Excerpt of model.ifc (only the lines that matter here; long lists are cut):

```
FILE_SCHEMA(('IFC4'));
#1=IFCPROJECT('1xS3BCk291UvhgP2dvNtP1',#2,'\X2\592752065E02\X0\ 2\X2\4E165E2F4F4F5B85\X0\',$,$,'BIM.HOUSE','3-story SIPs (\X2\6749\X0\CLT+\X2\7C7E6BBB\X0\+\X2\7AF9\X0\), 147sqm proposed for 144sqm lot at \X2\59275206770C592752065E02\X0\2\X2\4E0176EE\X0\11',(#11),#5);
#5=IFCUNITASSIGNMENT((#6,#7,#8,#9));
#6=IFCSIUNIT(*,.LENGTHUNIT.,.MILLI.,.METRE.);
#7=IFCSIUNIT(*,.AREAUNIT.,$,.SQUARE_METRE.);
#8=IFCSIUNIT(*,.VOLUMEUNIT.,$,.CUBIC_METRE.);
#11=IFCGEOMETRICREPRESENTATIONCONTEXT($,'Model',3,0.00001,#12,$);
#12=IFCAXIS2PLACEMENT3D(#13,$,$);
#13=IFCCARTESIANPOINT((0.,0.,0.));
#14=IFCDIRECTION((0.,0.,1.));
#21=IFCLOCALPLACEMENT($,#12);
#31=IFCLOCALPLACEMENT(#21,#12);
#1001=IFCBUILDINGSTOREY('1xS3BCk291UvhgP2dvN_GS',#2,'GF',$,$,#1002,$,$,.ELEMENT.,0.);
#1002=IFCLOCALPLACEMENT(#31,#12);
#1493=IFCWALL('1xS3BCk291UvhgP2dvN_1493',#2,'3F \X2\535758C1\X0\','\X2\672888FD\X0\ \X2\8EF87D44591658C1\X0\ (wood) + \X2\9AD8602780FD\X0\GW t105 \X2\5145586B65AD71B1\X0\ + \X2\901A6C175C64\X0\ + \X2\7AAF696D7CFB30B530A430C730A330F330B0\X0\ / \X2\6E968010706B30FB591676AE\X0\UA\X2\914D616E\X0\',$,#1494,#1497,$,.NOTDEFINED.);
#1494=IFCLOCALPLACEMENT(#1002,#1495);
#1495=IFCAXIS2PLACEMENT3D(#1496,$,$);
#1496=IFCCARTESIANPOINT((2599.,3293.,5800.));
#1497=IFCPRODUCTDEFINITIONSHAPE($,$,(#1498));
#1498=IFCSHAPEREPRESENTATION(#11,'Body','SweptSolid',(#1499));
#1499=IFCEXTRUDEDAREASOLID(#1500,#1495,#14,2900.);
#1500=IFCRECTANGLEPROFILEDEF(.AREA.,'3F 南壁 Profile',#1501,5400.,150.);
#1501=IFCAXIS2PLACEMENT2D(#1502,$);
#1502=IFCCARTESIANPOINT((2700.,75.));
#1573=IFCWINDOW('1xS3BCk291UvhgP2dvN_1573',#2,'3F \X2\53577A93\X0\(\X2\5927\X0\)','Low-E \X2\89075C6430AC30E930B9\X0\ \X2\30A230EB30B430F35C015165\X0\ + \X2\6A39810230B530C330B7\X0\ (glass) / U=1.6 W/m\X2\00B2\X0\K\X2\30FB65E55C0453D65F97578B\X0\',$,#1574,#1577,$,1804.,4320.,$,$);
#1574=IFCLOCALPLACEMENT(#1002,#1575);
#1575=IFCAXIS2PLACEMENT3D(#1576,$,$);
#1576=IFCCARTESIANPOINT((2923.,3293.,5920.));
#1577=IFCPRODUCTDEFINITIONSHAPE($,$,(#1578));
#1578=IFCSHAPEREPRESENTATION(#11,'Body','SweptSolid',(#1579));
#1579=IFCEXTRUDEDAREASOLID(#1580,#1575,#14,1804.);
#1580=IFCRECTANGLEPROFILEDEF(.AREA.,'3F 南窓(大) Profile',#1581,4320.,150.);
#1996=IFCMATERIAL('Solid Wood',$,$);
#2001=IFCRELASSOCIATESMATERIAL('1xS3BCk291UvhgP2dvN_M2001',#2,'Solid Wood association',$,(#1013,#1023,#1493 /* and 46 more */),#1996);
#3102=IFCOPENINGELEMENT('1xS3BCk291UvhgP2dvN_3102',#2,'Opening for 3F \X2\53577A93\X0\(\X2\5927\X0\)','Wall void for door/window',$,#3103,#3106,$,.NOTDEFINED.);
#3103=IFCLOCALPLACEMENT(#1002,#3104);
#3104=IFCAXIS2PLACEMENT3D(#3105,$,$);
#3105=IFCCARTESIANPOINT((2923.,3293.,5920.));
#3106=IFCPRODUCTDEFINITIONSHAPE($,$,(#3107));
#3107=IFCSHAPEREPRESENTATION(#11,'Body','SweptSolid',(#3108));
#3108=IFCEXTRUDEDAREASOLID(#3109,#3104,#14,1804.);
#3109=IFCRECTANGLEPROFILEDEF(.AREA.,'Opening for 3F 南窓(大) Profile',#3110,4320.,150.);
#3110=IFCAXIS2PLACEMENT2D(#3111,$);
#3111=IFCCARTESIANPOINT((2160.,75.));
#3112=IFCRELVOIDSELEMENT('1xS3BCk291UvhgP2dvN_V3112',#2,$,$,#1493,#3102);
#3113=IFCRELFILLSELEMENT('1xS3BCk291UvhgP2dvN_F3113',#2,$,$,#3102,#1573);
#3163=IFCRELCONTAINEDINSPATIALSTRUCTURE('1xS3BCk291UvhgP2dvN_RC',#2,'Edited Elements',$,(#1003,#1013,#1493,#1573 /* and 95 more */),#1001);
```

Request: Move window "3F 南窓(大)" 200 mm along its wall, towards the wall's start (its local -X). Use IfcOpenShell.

```python
import ifcopenshell
import ifcopenshell.api.geometry
import ifcopenshell.util.placement
import ifcopenshell.util.unit

model = ifcopenshell.open("model.ifc")
unit_scale = ifcopenshell.util.unit.calculate_unit_scale(model)

window = model.by_id(1573)
opening = window.FillsVoids[0].RelatingOpeningElement
wall = opening.VoidsElements[0].RelatingBuildingElement

wall_matrix = ifcopenshell.util.placement.get_local_placement(wall.ObjectPlacement)
shift = wall_matrix[:3, 0] * -0.2 / unit_scale
before = ifcopenshell.util.placement.get_local_placement(window.ObjectPlacement)[:3, 3].copy()

# The window is not placed relative to its opening, so move both.
for product in (opening, window):
    matrix = ifcopenshell.util.placement.get_local_placement(product.ObjectPlacement)
    matrix[:3, 3] += shift
    ifcopenshell.api.geometry.edit_object_placement(model, product=product, matrix=matrix, is_si=False)

after = ifcopenshell.util.placement.get_local_placement(window.ObjectPlacement)[:3, 3]
print("window moved by", (after - before).round(3) + 0.0)

model.write("model_edited.ifc")
```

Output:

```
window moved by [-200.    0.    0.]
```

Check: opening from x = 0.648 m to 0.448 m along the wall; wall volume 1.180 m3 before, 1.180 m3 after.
